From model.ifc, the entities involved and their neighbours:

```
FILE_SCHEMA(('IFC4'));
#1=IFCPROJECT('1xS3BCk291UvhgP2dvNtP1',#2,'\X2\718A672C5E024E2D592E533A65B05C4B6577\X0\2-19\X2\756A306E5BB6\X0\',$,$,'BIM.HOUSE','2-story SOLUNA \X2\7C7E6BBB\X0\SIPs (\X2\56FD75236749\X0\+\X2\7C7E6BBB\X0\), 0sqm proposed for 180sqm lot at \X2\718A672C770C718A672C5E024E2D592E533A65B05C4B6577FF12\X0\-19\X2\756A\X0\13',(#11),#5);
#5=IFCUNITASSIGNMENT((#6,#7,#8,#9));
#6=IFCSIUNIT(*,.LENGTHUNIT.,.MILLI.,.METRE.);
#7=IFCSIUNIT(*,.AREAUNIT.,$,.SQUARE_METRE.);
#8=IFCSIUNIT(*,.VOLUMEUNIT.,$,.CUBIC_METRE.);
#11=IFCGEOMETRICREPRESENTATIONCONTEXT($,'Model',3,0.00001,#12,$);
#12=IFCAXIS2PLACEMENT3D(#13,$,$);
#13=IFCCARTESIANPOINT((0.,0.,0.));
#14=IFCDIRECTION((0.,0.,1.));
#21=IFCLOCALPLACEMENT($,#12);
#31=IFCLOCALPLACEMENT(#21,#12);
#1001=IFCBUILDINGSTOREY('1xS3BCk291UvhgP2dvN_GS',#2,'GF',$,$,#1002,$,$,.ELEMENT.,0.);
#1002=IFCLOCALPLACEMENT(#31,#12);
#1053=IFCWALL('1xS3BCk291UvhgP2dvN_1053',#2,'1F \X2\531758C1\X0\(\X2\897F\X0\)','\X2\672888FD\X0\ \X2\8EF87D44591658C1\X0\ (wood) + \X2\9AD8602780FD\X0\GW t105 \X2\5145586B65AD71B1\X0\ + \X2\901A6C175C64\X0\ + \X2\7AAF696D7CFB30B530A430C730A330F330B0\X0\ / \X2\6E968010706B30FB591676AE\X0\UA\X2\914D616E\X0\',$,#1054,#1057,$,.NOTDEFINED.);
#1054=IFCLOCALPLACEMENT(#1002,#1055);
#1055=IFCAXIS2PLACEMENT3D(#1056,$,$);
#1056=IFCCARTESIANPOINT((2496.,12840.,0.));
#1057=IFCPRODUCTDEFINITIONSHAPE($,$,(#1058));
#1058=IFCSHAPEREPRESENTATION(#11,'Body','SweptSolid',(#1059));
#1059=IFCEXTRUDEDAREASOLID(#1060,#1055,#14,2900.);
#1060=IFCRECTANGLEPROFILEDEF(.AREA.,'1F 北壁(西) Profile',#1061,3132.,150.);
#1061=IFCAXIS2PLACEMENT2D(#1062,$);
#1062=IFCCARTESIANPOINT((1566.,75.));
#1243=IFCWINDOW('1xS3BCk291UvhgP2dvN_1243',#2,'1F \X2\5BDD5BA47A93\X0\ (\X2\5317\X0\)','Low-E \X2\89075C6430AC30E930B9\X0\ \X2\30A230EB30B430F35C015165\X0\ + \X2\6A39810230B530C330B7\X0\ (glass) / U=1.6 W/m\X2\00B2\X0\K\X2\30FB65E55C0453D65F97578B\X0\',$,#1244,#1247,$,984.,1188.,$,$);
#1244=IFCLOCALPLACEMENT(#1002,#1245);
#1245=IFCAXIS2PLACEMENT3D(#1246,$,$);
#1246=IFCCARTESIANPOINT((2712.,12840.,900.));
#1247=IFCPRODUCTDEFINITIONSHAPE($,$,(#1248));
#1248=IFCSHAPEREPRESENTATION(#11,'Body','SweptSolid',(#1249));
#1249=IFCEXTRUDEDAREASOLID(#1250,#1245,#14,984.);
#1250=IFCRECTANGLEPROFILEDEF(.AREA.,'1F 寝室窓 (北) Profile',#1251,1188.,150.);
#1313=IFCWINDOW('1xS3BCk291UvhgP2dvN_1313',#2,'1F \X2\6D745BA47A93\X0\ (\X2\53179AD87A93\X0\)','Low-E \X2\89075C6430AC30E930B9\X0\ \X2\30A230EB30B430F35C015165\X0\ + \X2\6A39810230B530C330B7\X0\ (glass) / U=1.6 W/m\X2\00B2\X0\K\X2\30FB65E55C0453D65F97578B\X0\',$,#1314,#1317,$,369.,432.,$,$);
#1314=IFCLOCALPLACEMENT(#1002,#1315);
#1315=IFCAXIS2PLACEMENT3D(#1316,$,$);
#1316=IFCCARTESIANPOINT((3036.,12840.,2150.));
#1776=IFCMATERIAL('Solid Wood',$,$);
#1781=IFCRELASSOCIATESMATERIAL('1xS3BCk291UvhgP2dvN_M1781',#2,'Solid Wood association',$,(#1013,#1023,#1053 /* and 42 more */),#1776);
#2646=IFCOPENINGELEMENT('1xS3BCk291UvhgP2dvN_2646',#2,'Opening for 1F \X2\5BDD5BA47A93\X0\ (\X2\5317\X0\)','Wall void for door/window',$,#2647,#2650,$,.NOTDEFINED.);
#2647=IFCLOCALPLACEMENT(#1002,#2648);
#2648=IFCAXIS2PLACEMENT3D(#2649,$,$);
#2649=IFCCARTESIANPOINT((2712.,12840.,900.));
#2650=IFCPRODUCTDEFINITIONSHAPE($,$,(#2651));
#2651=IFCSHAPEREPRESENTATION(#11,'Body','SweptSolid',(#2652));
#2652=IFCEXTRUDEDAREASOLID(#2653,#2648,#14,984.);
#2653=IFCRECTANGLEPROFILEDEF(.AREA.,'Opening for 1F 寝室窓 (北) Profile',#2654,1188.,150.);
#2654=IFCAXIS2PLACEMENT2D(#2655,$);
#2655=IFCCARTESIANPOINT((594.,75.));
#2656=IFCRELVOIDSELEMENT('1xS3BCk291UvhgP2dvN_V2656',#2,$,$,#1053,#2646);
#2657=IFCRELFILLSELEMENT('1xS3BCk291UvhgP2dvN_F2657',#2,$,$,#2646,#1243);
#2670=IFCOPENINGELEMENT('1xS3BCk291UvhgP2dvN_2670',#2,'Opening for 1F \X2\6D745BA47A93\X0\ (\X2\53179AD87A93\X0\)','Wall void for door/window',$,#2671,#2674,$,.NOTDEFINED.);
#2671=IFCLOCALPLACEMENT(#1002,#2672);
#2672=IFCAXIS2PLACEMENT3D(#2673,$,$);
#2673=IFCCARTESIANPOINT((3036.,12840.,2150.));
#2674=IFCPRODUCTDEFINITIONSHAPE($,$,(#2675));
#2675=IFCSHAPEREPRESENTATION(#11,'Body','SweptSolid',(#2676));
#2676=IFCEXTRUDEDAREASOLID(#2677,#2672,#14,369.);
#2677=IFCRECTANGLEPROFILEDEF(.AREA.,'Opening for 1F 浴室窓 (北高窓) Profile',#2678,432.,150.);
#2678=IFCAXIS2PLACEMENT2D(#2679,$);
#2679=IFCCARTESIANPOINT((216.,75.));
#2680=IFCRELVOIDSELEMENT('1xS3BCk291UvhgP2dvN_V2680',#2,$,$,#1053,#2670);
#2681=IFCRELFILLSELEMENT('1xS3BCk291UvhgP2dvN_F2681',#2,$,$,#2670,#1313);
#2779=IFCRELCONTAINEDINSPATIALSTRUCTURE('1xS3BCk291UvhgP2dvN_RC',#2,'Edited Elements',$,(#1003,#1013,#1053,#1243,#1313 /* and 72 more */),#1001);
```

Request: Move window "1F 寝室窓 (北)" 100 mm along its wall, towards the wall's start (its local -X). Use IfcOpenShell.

```python
import ifcopenshell
import ifcopenshell.api.geometry
import ifcopenshell.util.placement

model = ifcopenshell.open("model.ifc")

window = model.by_guid("1xS3BCk291UvhgP2dvN_1243")
opening = window.FillsVoids[0].RelatingOpeningElement
wall = opening.VoidsElements[0].RelatingBuildingElement

wall_matrix = ifcopenshell.util.placement.get_local_placement(wall.ObjectPlacement)
shift = wall_matrix[:3, 0] * -100.0
before = ifcopenshell.util.placement.get_local_placement(window.ObjectPlacement)[:3, 3].copy()

# The window is not placed relative to its opening, so move both.
for product in (opening, window):
    matrix = ifcopenshell.util.placement.get_local_placement(product.ObjectPlacement)
    matrix[:3, 3] += shift
    ifcopenshell.api.geometry.edit_object_placement(model, product=product, matrix=matrix, is_si=False)

after = ifcopenshell.util.placement.get_local_placement(window.ObjectPlacement)[:3, 3]
print("window moved by", (after - before).round(3) + 0.0)

model.write("model-out.ifc")
```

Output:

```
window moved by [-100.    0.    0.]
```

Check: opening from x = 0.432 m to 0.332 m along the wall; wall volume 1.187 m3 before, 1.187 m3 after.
